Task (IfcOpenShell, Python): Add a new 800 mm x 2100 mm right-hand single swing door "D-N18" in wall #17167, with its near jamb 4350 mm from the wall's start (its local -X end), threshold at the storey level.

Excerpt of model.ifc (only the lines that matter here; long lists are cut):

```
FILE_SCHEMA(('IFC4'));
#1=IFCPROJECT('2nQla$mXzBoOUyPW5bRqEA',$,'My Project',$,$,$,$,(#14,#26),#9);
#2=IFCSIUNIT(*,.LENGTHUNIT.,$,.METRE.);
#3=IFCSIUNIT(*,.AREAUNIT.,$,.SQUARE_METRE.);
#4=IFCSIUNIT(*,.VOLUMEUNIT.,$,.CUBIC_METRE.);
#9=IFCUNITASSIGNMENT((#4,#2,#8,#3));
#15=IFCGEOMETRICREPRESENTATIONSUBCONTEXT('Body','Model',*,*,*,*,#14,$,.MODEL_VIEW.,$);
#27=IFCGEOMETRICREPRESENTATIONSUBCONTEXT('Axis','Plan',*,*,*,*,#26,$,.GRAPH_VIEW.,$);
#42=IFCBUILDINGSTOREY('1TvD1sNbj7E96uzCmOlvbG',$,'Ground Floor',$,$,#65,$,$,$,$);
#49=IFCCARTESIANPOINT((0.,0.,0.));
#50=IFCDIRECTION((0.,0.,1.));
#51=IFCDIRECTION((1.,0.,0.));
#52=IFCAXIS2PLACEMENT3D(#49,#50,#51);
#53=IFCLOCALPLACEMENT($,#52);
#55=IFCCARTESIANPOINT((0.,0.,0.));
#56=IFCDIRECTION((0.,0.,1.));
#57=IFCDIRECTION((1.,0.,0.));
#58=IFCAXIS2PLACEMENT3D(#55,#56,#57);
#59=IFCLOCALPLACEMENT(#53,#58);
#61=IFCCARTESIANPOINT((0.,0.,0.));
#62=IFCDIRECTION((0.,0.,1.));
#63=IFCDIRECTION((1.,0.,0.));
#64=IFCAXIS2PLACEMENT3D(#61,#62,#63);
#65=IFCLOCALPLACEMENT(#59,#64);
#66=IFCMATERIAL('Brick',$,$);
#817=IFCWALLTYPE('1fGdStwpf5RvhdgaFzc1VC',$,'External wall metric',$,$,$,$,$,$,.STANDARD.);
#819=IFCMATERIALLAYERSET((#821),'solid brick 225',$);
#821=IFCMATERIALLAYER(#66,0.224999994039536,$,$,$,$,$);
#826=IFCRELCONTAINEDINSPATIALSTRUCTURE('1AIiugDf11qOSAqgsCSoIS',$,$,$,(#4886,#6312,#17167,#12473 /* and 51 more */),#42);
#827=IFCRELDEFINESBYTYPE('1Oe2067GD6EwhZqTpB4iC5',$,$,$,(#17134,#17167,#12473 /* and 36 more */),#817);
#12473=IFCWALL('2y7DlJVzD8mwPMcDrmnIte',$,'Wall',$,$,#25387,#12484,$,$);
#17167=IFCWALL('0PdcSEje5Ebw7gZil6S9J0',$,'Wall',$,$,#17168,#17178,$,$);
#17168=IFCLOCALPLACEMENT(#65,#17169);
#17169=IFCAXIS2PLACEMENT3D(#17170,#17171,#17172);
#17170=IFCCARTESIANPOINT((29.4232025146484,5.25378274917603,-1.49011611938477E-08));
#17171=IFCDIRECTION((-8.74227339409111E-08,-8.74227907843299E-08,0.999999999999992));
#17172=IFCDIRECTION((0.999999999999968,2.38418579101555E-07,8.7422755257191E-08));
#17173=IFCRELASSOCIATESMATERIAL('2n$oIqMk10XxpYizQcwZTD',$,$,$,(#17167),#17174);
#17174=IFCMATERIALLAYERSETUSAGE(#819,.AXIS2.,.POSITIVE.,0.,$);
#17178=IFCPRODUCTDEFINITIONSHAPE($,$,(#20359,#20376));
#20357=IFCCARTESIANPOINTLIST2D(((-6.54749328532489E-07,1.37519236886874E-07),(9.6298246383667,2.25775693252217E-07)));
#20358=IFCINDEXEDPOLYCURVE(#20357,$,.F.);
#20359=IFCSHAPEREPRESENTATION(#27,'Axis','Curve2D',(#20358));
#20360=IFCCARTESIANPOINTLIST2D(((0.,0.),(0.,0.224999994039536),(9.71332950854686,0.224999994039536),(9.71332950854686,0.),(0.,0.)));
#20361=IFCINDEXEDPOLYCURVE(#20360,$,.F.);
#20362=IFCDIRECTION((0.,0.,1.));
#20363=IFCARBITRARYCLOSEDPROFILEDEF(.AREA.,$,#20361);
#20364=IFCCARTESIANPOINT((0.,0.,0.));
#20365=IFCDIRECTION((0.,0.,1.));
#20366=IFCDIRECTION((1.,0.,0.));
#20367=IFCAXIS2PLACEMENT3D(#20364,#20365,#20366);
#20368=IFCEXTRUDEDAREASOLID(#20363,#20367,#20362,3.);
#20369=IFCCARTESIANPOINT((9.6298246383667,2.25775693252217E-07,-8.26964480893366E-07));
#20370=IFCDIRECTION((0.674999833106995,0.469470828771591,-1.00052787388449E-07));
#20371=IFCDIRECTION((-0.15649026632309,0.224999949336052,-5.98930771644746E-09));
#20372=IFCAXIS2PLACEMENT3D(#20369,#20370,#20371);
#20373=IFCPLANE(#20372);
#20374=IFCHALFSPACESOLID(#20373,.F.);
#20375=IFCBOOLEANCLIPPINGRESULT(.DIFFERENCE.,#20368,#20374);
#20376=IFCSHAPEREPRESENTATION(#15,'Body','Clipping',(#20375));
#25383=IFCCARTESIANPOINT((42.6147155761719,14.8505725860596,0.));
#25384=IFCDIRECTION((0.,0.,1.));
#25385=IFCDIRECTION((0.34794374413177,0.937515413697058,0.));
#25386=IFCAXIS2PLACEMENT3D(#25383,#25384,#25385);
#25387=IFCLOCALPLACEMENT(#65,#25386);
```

```python
import numpy as np
import ifcopenshell
import ifcopenshell.api.feature
import ifcopenshell.api.geometry
import ifcopenshell.api.root
import ifcopenshell.api.spatial
import ifcopenshell.geom
import ifcopenshell.util.element
import ifcopenshell.util.placement
import ifcopenshell.util.representation
import ifcopenshell.util.shape
import ifcopenshell.util.unit

model = ifcopenshell.open("model.ifc")
unit_scale = ifcopenshell.util.unit.calculate_unit_scale(model)
settings = ifcopenshell.geom.settings()


def volume(element):
    """Net volume in cubic metres, openings subtracted."""
    shape = ifcopenshell.geom.create_shape(settings, element)
    return ifcopenshell.util.shape.get_volume(shape.geometry)


wall = model.by_guid("0PdcSEje5Ebw7gZil6S9J0")
storey = ifcopenshell.util.element.get_container(wall, ifc_class="IfcBuildingStorey")
context = ifcopenshell.util.representation.get_context(model, "Model", "Body", "MODEL_VIEW")
before = volume(wall)

width, height, from_end, sill = 0.8, 2.1, 4.35, 0.0  # metres

# The wall runs along its own X axis, and the end named is its -X end.
wall_shape = ifcopenshell.geom.create_shape(settings, wall)
x, y, z = ifcopenshell.util.shape.get_vertices(wall_shape.geometry).T
start = x.min() + from_end
face, thickness = float(y.min()), float(y.max() - y.min())
wall_matrix = ifcopenshell.util.placement.get_local_placement(wall.ObjectPlacement)
level = ifcopenshell.util.placement.get_local_placement(storey.ObjectPlacement)[2, 3]


def in_wall(x, y):
    """Placement at x, y metres in the wall's axes, at sill height."""
    matrix = wall_matrix.copy()
    matrix[:, 3] = wall_matrix @ np.array([x / unit_scale, y / unit_scale, 0.0, 1.0])
    matrix[2, 3] = level + sill / unit_scale
    return matrix


# Opening: a box that overshoots both wall faces by 50 mm.
opening = ifcopenshell.api.root.create_entity(model, ifc_class="IfcOpeningElement", predefined_type="OPENING")
box = ifcopenshell.api.geometry.add_wall_representation(
    model, context=context, length=width, height=height, thickness=thickness + 0.1
)
ifcopenshell.api.geometry.assign_representation(model, product=opening, representation=box)
ifcopenshell.api.geometry.edit_object_placement(model, product=opening, matrix=in_wall(start, face - 0.05), is_si=False)
ifcopenshell.api.feature.add_feature(model, feature=opening, element=wall)

door = ifcopenshell.api.root.create_entity(model, ifc_class="IfcDoor", name="D-N18", predefined_type="DOOR")
door.OverallWidth, door.OverallHeight = width / unit_scale, height / unit_scale
door.OperationType = "SINGLE_SWING_RIGHT"
body = ifcopenshell.api.geometry.add_door_representation(
    model,
    context=context,
    overall_width=door.OverallWidth,
    overall_height=door.OverallHeight,
    operation_type="SINGLE_SWING_RIGHT",
    lining_properties={"LiningDepth": thickness / unit_scale, "ThresholdDepth": thickness / unit_scale},
)
ifcopenshell.api.geometry.assign_representation(model, product=door, representation=body)
ifcopenshell.api.spatial.assign_container(model, products=[door], relating_structure=storey)
ifcopenshell.api.feature.add_filling(model, opening=opening, element=door)

# The lining spans the wall, so the door starts at the wall face.
ifcopenshell.api.geometry.edit_object_placement(model, product=door, matrix=in_wall(start, face), is_si=False)

after = volume(wall)

print(f"wall volume {before:.3f} -> {after:.3f} m3")

model.write("model_rev.ifc")
```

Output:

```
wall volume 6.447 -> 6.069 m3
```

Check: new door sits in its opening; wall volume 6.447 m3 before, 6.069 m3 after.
